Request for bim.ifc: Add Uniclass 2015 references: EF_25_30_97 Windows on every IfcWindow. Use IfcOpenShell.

First a look at what the model holds.

```python
import ifcopenshell

model = ifcopenshell.open("bim.ifc")
print(model.schema)
print("classifications:", [c.Name for c in model.by_type("IfcClassification")])
for ifc_class in ("IfcDoor", "IfcRoof", "IfcStair", "IfcWall", "IfcWindow"):
    print(ifc_class, len(model.by_type(ifc_class)))
```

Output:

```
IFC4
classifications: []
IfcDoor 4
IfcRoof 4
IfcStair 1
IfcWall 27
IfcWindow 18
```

```python
import ifcopenshell
import ifcopenshell.api.classification

model = ifcopenshell.open("bim.ifc")

system = ifcopenshell.api.classification.add_classification(model, classification="Uniclass 2015")

codes = {
    "IfcWindow": ("EF_25_30_97", "Windows"),
}
for ifc_class, (code, name) in codes.items():
    products = model.by_type(ifc_class)
    ifcopenshell.api.classification.add_reference(
        model, products=products, classification=system, identification=code, name=name
    )
    print(code, len(products))

model.write("bim_edited.ifc")
```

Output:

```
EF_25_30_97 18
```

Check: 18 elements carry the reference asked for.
